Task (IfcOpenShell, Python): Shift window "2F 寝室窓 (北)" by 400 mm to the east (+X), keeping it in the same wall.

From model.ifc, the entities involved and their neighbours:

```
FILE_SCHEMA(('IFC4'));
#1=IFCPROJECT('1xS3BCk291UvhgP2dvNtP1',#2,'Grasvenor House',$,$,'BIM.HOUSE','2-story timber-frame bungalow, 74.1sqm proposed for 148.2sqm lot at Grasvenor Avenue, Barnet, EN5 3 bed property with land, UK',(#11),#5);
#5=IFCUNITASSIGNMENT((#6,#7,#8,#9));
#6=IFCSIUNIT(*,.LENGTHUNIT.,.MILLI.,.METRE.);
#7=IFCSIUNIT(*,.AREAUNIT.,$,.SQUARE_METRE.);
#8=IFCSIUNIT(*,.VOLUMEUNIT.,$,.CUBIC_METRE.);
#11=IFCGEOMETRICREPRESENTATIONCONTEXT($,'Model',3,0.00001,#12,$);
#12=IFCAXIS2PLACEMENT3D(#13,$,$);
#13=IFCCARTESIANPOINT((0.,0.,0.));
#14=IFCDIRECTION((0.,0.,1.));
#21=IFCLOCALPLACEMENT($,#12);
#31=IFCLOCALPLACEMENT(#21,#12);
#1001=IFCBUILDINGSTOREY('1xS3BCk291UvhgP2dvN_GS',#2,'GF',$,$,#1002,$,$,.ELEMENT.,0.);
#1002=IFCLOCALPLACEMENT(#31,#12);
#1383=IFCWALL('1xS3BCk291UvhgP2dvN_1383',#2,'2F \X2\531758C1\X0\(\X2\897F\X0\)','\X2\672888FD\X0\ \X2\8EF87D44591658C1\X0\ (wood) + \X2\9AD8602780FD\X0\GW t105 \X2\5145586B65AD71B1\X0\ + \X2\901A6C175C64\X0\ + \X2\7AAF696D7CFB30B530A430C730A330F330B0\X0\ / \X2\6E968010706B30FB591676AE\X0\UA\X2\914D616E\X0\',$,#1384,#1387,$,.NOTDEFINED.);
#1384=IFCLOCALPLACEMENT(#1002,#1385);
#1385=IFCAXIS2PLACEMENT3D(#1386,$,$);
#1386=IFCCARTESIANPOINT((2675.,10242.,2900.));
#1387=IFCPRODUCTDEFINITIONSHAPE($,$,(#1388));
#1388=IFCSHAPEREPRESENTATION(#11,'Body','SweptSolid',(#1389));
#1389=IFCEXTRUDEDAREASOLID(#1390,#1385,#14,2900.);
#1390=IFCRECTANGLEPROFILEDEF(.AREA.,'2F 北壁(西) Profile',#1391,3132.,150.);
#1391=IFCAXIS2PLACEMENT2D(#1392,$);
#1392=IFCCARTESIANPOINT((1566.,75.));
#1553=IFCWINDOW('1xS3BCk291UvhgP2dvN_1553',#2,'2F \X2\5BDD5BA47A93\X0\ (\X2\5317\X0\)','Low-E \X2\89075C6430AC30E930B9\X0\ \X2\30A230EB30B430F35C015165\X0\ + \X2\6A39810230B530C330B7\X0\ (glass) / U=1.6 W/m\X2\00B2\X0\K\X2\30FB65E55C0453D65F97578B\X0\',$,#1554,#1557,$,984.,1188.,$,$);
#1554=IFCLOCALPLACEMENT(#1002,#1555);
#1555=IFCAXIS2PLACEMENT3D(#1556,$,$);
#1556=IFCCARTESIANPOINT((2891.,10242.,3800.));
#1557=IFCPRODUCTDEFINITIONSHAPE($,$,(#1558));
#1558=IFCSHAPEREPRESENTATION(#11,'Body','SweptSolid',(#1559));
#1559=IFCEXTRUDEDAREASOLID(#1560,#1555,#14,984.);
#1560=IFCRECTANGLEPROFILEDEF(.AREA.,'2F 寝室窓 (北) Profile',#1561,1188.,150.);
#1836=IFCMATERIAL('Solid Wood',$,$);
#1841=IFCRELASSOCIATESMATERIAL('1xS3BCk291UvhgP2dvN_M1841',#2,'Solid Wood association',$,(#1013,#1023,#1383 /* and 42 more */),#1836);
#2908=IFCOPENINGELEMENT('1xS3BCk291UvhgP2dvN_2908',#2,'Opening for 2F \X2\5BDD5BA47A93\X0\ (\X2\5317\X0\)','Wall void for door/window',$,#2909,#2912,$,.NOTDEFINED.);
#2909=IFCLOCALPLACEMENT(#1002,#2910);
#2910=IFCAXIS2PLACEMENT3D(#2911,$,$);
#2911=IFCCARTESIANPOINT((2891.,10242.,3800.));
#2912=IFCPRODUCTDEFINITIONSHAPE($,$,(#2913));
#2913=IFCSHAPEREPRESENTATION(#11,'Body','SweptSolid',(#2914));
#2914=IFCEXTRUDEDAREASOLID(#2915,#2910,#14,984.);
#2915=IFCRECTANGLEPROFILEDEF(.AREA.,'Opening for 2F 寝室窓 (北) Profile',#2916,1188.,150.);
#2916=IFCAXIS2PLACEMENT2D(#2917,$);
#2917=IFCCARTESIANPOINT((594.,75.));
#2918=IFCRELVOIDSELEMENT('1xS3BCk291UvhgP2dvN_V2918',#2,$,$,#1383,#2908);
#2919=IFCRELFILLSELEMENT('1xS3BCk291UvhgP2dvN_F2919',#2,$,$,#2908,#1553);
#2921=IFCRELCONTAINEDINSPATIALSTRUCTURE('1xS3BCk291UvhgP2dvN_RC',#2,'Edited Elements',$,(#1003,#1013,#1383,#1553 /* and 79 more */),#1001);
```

```python
import ifcopenshell
import ifcopenshell.api.geometry
import ifcopenshell.util.placement
import ifcopenshell.util.unit

model = ifcopenshell.open("model.ifc")
unit_scale = ifcopenshell.util.unit.calculate_unit_scale(model)

window = model.by_guid("1xS3BCk291UvhgP2dvN_1553")
opening = window.FillsVoids[0].RelatingOpeningElement
wall = opening.VoidsElements[0].RelatingBuildingElement

wall_matrix = ifcopenshell.util.placement.get_local_placement(wall.ObjectPlacement)
shift = wall_matrix[:3, 0] * 0.4 / unit_scale
before = ifcopenshell.util.placement.get_local_placement(window.ObjectPlacement)[:3, 3].copy()

# The window is not placed relative to its opening, so move both.
for product in (opening, window):
    matrix = ifcopenshell.util.placement.get_local_placement(product.ObjectPlacement)
    matrix[:3, 3] += shift
    ifcopenshell.api.geometry.edit_object_placement(model, product=product, matrix=matrix, is_si=False)

after = ifcopenshell.util.placement.get_local_placement(window.ObjectPlacement)[:3, 3]
print("window moved by", (after - before).round(3) + 0.0)

model.write("model_rev.ifc")
```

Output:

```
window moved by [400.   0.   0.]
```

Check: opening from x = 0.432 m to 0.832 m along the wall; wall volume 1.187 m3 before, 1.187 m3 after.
